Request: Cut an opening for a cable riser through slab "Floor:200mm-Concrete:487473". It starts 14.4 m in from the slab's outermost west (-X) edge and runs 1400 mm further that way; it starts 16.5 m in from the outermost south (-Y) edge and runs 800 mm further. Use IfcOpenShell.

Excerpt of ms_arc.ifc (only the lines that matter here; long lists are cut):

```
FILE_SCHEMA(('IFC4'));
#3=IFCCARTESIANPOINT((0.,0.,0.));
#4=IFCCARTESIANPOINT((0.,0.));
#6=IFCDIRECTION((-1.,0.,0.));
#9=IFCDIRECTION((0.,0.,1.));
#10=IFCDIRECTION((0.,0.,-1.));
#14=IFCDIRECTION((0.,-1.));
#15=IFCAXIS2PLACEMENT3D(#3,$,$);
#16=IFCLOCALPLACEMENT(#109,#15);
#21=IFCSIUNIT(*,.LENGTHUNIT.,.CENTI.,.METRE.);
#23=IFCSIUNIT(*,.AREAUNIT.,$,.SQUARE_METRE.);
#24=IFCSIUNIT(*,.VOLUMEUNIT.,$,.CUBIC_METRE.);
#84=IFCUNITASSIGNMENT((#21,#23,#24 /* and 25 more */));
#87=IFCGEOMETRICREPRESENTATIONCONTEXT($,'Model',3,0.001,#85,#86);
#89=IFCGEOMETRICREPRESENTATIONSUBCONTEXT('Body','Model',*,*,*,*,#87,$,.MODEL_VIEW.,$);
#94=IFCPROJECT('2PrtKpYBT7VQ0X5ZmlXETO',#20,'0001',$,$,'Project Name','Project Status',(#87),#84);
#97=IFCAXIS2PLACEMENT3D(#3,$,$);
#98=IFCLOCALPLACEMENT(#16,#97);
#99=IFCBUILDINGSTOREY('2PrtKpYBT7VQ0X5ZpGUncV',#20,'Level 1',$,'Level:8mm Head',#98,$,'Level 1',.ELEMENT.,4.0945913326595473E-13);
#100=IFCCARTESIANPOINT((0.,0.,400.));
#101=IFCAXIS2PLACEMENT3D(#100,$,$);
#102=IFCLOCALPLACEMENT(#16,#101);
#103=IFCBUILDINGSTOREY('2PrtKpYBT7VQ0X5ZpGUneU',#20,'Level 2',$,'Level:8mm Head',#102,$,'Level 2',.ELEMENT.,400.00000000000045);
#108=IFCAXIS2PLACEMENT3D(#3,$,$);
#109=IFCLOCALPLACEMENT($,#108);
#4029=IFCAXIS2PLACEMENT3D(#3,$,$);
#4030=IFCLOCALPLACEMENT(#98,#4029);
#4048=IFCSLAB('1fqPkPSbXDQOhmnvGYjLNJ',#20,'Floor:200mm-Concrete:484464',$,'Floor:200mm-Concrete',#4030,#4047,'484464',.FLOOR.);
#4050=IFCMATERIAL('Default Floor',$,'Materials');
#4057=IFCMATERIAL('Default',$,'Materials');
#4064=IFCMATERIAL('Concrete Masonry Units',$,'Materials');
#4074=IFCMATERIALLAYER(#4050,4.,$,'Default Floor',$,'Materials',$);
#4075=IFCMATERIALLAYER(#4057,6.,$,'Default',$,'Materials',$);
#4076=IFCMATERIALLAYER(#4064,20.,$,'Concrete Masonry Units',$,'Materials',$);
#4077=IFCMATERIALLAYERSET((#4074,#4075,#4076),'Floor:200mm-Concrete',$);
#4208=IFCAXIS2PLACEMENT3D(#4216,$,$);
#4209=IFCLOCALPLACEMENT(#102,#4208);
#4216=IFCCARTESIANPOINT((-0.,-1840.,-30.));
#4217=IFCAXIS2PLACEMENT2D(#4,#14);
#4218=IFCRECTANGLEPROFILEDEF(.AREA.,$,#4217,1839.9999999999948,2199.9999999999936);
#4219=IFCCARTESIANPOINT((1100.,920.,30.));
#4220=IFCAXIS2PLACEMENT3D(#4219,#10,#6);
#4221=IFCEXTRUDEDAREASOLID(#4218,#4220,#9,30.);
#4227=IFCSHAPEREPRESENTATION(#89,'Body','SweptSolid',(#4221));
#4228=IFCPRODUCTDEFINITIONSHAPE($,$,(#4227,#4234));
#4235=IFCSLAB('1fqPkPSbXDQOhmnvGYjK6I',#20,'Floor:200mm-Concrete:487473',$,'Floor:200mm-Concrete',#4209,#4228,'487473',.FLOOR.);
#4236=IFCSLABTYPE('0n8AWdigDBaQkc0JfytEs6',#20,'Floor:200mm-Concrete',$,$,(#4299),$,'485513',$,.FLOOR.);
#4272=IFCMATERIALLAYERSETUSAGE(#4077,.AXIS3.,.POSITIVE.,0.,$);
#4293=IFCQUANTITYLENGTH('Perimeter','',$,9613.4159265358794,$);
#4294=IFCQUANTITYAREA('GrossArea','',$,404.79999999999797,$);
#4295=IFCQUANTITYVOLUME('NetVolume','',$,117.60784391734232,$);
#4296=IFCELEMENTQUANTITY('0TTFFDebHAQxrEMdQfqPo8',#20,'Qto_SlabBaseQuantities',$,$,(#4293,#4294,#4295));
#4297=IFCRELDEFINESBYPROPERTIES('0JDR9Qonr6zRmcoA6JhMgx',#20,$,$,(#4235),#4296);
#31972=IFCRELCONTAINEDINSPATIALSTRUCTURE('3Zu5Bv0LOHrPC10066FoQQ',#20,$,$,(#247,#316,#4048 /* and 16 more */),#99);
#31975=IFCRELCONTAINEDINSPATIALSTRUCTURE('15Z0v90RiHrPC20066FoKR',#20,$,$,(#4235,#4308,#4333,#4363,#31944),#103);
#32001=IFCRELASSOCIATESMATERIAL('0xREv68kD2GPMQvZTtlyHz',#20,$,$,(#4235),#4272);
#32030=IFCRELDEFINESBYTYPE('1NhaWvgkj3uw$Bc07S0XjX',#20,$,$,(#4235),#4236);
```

```python
import numpy as np
import ifcopenshell
import ifcopenshell.api.feature
import ifcopenshell.api.geometry
import ifcopenshell.api.pset
import ifcopenshell.api.root
import ifcopenshell.geom
import ifcopenshell.util.element
import ifcopenshell.util.placement
import ifcopenshell.util.representation
import ifcopenshell.util.shape
import ifcopenshell.util.unit

model = ifcopenshell.open("ms_arc.ifc")
unit_scale = ifcopenshell.util.unit.calculate_unit_scale(model)
volume_scale = ifcopenshell.util.unit.calculate_unit_scale(model, "VOLUMEUNIT")
settings = ifcopenshell.geom.settings()


def volume(element):
    """Net volume in cubic metres, openings subtracted."""
    shape = ifcopenshell.geom.create_shape(settings, element)
    return ifcopenshell.util.shape.get_volume(shape.geometry)


slab = model.by_guid("1fqPkPSbXDQOhmnvGYjK6I")
before = volume(slab)

# Extent in the slab's own axes, in metres. The edges named are its -X and -Y sides.
slab_shape = ifcopenshell.geom.create_shape(settings, slab)
vertices = ifcopenshell.util.shape.get_vertices(slab_shape.geometry)
x_min, y_min, bottom = vertices.min(axis=0)
top = vertices[:, 2].max()

opening = ifcopenshell.api.root.create_entity(model, ifc_class="IfcOpeningElement", name="Cable riser opening", predefined_type="OPENING")
context = ifcopenshell.util.representation.get_context(model, "Model", "Body", "MODEL_VIEW")
width, depth = 1.4, 0.8
outline = [(0.0, 0.0), (width, 0.0), (width, depth), (0.0, depth), (0.0, 0.0)]
# Overshoot both faces by 50 mm so the cut is clean.
shape = ifcopenshell.api.geometry.add_slab_representation(
    model, context=context, depth=top - bottom + 0.1, polyline=outline
)
ifcopenshell.api.geometry.assign_representation(model, product=opening, representation=shape)

matrix = ifcopenshell.util.placement.get_local_placement(slab.ObjectPlacement)
matrix[:, 3] = matrix @ np.append(np.array([x_min + 14.4, y_min + 16.5, bottom - 0.05]) / unit_scale, 1.0)
ifcopenshell.api.geometry.edit_object_placement(model, product=opening, matrix=matrix, is_si=False)
ifcopenshell.api.feature.add_feature(model, feature=opening, element=slab)

after = volume(slab)

# Update the slab's stored quantities.
qto = model.by_id(ifcopenshell.util.element.get_pset(slab, "Qto_SlabBaseQuantities", should_inherit=False)["id"])
ifcopenshell.api.pset.edit_qto(model, qto=qto, properties={"NetVolume": after / volume_scale})

print(f"slab volume {before:.3f} -> {after:.3f} m3")

model.write("ms_arc_v2.ifc")
```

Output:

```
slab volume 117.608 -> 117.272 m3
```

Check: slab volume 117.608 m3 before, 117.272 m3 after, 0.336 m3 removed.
